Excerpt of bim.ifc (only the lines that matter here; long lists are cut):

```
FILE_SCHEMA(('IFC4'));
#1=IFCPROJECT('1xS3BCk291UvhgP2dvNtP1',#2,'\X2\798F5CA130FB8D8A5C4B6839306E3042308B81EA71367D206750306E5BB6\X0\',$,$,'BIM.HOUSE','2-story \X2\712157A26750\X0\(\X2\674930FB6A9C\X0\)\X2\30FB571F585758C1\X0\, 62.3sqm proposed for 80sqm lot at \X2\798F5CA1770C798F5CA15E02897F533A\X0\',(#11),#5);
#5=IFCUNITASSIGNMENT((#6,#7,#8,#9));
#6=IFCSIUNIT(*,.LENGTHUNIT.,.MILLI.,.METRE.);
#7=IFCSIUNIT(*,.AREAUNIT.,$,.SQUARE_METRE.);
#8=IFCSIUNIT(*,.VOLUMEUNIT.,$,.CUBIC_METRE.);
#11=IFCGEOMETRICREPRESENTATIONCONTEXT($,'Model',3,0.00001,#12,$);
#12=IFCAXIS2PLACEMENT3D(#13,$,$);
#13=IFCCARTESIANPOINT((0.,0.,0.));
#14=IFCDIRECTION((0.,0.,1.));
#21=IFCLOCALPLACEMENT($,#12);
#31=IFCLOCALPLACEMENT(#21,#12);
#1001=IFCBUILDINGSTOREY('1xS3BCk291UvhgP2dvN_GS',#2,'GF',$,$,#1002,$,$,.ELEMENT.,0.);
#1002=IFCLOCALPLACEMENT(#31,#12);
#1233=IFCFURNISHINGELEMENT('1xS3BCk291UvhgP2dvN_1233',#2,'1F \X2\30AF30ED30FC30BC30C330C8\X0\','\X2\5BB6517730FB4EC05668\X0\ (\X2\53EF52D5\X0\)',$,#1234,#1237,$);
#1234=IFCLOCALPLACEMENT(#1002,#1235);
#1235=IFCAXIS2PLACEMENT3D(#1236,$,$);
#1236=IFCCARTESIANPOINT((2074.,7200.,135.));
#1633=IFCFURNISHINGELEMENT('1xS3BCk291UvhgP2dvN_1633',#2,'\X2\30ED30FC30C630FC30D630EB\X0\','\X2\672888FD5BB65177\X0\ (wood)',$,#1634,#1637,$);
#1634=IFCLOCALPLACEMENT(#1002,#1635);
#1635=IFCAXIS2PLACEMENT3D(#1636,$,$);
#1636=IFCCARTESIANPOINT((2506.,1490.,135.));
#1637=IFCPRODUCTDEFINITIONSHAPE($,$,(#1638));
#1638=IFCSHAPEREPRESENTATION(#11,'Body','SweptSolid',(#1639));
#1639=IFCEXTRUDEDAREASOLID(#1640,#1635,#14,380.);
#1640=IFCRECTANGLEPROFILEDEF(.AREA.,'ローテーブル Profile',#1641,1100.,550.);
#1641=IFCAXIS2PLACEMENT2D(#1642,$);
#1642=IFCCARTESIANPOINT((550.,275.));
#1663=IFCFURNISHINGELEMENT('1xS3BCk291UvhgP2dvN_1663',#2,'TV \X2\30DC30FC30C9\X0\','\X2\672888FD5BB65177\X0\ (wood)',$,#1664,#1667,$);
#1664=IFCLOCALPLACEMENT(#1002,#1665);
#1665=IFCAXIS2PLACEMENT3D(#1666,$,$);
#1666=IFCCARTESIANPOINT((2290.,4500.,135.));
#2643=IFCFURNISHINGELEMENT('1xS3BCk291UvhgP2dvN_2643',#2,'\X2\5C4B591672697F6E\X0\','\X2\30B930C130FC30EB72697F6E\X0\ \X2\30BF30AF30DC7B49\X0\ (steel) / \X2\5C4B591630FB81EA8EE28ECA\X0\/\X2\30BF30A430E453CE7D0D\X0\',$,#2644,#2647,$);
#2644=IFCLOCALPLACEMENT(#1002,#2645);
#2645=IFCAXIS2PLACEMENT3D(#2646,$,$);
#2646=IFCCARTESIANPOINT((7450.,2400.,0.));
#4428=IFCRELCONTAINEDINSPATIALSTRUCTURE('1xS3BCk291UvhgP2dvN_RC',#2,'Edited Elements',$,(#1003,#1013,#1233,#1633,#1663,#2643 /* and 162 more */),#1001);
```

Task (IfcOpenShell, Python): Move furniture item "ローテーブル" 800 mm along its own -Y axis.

```python
import ifcopenshell
import ifcopenshell.api.geometry
import ifcopenshell.util.placement

model = ifcopenshell.open("bim.ifc")

item = model.by_guid("1xS3BCk291UvhgP2dvN_1633")
matrix = ifcopenshell.util.placement.get_local_placement(item.ObjectPlacement)
matrix[:3, 3] -= matrix[:3, 1] * 800.0
ifcopenshell.api.geometry.edit_object_placement(model, product=item, matrix=matrix, is_si=False)

print(ifcopenshell.util.placement.get_local_placement(item.ObjectPlacement).round(3) + 0.0)

model.write("bim_edited.ifc")
```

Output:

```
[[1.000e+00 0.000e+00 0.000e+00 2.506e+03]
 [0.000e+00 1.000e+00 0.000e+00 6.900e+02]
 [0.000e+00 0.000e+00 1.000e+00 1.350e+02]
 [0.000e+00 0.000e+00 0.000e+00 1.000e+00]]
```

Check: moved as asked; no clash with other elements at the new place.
